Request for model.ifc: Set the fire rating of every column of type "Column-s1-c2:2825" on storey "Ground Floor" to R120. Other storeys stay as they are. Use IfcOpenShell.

First a look at what the model holds.

```python
import ifcopenshell
import ifcopenshell.util.element

model = ifcopenshell.open("model.ifc")
print(model.schema)
storey = next(s for s in model.by_type("IfcBuildingStorey") if s.Name == "Ground Floor")
columns = [e for e in ifcopenshell.util.element.get_decomposition(storey) if e.is_a("IfcColumn")]
seen = {}
for e in columns:
    element_type = ifcopenshell.util.element.get_type(e)
    key = (element_type.Name if element_type != e and element_type else None, ifcopenshell.util.element.get_pset(e, "Pset_ColumnCommon", "FireRating"))
    seen[key] = seen.get(key, 0) + 1
for (name, value), count in sorted(seen.items(), key=str):
    print(count, "x", name, "|", value)
```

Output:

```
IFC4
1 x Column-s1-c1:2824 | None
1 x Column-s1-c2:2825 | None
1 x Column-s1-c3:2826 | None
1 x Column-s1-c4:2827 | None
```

```python
import ifcopenshell
import ifcopenshell.api.pset
import ifcopenshell.util.element

model = ifcopenshell.open("model.ifc")

storey = next(s for s in model.by_type("IfcBuildingStorey") if s.Name == "Ground Floor")
columns = [e for e in ifcopenshell.util.element.get_decomposition(storey) if e.is_a("IfcColumn")]

count = 0
for e in columns:
    element_type = ifcopenshell.util.element.get_type(e)
    if element_type in (None, e) or element_type.Name != "Column-s1-c2:2825":
        continue
    # add_pset returns the element's existing set when there is one.
    pset = ifcopenshell.api.pset.add_pset(model, product=e, name="Pset_ColumnCommon")
    ifcopenshell.api.pset.edit_pset(model, pset=pset, properties={"FireRating": "R120"})
    count += 1

print(count, "columns updated")

model.write("model_updated.ifc")
```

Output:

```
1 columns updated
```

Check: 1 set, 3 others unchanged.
